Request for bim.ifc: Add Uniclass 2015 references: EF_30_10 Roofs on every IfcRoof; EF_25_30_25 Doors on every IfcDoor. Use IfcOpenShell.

First a look at what the model holds.

```python
import ifcopenshell

model = ifcopenshell.open("bim.ifc")
print(model.schema)
print("classifications:", [c.Name for c in model.by_type("IfcClassification")])
for ifc_class in ("IfcDoor", "IfcRoof", "IfcStair", "IfcWall", "IfcWindow"):
    print(ifc_class, len(model.by_type(ifc_class)))
```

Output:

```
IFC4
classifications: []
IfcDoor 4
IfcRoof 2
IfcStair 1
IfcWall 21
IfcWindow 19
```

```python
import ifcopenshell
import ifcopenshell.api.classification

model = ifcopenshell.open("bim.ifc")

system = ifcopenshell.api.classification.add_classification(model, classification="Uniclass 2015")

codes = {
    "IfcRoof": ("EF_30_10", "Roofs"),
    "IfcDoor": ("EF_25_30_25", "Doors"),
}
for ifc_class, (code, name) in codes.items():
    products = model.by_type(ifc_class)
    ifcopenshell.api.classification.add_reference(
        model, products=products, classification=system, identification=code, name=name
    )
    print(code, len(products))

model.write("bim_v2.ifc")
```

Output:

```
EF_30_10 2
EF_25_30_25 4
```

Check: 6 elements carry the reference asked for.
